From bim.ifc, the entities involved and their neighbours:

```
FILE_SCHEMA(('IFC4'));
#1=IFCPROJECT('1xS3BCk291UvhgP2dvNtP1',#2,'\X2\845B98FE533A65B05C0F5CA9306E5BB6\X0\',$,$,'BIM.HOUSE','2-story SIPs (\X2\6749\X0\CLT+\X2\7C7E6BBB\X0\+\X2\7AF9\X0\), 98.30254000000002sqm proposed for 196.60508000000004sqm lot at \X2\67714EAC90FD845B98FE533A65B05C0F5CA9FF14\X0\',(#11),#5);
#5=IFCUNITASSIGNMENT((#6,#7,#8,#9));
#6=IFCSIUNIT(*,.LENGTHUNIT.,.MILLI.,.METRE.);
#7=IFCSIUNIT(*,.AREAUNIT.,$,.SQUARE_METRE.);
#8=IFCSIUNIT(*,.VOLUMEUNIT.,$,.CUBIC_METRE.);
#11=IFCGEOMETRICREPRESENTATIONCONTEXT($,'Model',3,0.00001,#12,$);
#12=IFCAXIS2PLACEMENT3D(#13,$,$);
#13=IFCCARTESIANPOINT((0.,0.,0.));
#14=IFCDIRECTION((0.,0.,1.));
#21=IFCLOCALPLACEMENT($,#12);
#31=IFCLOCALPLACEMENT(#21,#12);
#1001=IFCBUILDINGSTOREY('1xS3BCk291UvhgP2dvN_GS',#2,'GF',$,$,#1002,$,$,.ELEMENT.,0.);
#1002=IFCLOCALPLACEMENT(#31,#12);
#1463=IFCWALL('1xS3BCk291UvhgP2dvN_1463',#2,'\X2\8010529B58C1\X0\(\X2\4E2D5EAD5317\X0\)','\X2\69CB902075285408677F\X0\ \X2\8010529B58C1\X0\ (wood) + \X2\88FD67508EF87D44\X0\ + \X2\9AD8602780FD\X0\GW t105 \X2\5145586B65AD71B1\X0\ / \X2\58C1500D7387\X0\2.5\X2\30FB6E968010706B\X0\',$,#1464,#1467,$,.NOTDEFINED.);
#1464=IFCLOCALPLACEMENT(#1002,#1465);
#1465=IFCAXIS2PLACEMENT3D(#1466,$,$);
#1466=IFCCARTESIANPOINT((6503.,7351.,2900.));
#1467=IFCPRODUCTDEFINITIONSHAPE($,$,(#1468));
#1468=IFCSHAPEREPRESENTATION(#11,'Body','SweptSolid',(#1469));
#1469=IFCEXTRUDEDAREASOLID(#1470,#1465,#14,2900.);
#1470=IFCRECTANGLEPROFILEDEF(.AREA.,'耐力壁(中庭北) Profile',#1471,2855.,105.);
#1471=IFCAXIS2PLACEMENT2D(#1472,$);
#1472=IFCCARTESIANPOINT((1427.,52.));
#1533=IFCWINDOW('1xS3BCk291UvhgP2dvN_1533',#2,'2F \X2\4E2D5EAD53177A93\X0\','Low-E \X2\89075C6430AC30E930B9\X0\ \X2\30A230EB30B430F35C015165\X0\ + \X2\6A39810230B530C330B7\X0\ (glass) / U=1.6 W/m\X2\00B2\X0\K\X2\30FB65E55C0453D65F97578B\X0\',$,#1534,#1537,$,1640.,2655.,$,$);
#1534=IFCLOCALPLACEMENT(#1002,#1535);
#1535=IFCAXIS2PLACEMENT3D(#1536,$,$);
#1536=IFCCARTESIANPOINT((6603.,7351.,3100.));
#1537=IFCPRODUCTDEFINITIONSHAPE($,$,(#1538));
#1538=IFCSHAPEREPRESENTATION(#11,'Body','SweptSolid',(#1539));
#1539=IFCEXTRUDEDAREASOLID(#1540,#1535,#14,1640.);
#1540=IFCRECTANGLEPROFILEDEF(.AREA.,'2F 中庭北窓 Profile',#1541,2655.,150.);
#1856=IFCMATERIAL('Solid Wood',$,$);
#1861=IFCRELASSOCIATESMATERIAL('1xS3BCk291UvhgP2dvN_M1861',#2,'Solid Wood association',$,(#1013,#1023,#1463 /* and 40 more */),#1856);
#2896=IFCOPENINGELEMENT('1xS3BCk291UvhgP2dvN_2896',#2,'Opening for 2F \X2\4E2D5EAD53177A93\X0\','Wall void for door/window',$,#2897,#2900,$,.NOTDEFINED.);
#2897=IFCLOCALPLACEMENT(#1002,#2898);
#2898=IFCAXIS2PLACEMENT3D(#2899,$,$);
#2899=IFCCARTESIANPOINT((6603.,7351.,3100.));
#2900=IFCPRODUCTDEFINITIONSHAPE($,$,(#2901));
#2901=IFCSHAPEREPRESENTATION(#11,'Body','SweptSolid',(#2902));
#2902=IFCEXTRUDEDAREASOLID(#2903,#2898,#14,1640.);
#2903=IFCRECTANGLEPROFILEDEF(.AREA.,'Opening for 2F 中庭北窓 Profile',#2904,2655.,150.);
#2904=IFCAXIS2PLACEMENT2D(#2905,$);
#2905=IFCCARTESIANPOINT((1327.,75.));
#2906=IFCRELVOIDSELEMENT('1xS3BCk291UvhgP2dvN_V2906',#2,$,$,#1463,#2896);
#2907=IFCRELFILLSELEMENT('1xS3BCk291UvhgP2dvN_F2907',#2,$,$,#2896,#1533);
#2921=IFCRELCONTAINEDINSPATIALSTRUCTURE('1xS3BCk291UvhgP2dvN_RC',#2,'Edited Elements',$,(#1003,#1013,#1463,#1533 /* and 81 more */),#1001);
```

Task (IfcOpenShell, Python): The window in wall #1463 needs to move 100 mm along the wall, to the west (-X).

```python
import ifcopenshell
import ifcopenshell.api.geometry
import ifcopenshell.util.placement
import ifcopenshell.util.unit

model = ifcopenshell.open("bim.ifc")
unit_scale = ifcopenshell.util.unit.calculate_unit_scale(model)

window = model.by_guid("1xS3BCk291UvhgP2dvN_1533")
opening = window.FillsVoids[0].RelatingOpeningElement
wall = opening.VoidsElements[0].RelatingBuildingElement

wall_matrix = ifcopenshell.util.placement.get_local_placement(wall.ObjectPlacement)
shift = wall_matrix[:3, 0] * -0.1 / unit_scale
before = ifcopenshell.util.placement.get_local_placement(window.ObjectPlacement)[:3, 3].copy()

# The window is not placed relative to its opening, so move both.
for product in (opening, window):
    matrix = ifcopenshell.util.placement.get_local_placement(product.ObjectPlacement)
    matrix[:3, 3] += shift
    ifcopenshell.api.geometry.edit_object_placement(model, product=product, matrix=matrix, is_si=False)

after = ifcopenshell.util.placement.get_local_placement(window.ObjectPlacement)[:3, 3]
print("window moved by", (after - before).round(3) + 0.0)

model.write("bim-out.ifc")
```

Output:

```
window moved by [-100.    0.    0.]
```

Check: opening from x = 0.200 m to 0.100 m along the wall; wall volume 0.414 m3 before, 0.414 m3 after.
